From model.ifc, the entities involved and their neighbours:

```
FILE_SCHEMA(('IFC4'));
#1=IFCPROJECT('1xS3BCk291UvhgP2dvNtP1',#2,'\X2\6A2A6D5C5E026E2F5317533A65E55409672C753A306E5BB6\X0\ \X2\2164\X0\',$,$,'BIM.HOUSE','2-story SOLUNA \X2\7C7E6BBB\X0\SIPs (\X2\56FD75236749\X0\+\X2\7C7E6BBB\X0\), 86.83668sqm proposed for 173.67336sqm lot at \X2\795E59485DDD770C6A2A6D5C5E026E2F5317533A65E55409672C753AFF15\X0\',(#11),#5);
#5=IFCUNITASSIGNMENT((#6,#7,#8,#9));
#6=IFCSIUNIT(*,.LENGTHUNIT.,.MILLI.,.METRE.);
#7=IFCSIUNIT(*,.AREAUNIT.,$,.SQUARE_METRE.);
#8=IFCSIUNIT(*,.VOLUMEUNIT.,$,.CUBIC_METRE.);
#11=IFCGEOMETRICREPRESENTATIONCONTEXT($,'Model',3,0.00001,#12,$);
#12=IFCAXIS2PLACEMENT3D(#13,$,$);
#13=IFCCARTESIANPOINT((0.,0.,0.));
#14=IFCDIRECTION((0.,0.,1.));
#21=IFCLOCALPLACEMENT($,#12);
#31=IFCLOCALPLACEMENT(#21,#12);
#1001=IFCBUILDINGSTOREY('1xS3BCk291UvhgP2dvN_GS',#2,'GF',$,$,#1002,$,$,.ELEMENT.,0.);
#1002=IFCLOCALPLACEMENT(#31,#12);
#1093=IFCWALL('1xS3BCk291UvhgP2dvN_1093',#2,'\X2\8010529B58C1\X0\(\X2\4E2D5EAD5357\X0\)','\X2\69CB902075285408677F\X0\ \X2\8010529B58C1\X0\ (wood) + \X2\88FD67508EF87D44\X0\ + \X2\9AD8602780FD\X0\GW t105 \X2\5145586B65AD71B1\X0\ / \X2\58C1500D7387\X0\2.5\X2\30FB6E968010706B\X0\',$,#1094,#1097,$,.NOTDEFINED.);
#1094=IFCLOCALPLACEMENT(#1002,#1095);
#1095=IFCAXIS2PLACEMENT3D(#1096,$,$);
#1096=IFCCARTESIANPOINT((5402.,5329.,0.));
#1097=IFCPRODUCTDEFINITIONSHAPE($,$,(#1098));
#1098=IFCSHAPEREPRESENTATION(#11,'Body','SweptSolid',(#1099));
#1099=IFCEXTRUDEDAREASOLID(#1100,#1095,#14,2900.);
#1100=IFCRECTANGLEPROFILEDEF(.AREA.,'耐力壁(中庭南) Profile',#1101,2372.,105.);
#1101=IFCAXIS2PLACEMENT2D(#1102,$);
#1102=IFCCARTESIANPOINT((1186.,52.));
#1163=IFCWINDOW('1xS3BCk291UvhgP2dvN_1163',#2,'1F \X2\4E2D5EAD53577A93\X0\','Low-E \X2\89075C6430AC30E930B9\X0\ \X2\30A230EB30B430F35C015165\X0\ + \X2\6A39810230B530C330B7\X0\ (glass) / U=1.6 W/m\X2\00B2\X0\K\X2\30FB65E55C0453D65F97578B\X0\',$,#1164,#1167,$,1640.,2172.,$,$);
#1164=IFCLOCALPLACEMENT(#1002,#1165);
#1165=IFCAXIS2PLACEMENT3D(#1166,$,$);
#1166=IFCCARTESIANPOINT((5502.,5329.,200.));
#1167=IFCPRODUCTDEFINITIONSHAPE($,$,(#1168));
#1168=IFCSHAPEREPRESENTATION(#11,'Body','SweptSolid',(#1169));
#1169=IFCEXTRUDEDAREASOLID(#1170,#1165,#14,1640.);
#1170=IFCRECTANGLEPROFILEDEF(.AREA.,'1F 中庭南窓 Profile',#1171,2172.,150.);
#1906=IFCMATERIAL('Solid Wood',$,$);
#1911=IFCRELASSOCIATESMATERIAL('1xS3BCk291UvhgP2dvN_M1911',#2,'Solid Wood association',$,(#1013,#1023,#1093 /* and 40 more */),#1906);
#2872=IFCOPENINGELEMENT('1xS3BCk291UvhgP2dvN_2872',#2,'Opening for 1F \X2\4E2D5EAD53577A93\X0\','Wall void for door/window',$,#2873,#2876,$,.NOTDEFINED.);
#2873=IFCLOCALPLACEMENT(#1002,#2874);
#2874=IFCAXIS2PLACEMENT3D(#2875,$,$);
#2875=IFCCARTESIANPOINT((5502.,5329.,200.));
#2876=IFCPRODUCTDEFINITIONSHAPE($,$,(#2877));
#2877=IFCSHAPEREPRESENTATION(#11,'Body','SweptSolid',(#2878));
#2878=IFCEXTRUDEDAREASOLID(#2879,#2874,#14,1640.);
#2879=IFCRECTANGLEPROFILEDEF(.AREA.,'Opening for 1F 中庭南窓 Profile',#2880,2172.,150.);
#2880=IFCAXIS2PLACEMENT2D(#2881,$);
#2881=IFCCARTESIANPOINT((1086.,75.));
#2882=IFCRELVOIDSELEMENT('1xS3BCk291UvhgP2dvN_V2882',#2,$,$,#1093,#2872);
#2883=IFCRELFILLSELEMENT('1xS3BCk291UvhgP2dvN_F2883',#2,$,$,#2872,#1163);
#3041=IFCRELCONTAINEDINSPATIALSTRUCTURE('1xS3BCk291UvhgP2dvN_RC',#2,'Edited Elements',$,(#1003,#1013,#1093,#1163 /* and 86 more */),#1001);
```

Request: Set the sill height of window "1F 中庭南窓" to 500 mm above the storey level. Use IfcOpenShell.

```python
import numpy as np
import ifcopenshell
import ifcopenshell.api.geometry
import ifcopenshell.geom
import ifcopenshell.util.element
import ifcopenshell.util.placement
import ifcopenshell.util.shape
import ifcopenshell.util.unit

model = ifcopenshell.open("model.ifc")
unit_scale = ifcopenshell.util.unit.calculate_unit_scale(model)

window = model.by_guid("1xS3BCk291UvhgP2dvN_1163")
opening = window.FillsVoids[0].RelatingOpeningElement
storey = ifcopenshell.util.element.get_container(window, ifc_class="IfcBuildingStorey")
level = ifcopenshell.util.placement.get_local_placement(storey.ObjectPlacement)[2, 3]

# The opening's origin need not be at the sill, so measure its lowest point.
shape = ifcopenshell.geom.create_shape(ifcopenshell.geom.settings(), opening)
bottom = ifcopenshell.util.shape.get_shape_bottom_elevation(shape, shape.geometry) / unit_scale
dz = level + 0.5 / unit_scale - bottom

shift = np.array([0.0, 0.0, dz])
# The window is not placed relative to its opening, so move both.
for product in (opening, window):
    matrix = ifcopenshell.util.placement.get_local_placement(product.ObjectPlacement)
    matrix[:3, 3] += shift
    ifcopenshell.api.geometry.edit_object_placement(model, product=product, matrix=matrix, is_si=False)

print(f"moved by {dz * unit_scale:+.3f} m")

model.write("model_edited.ifc")
```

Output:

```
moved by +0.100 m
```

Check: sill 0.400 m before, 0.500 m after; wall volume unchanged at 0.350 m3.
